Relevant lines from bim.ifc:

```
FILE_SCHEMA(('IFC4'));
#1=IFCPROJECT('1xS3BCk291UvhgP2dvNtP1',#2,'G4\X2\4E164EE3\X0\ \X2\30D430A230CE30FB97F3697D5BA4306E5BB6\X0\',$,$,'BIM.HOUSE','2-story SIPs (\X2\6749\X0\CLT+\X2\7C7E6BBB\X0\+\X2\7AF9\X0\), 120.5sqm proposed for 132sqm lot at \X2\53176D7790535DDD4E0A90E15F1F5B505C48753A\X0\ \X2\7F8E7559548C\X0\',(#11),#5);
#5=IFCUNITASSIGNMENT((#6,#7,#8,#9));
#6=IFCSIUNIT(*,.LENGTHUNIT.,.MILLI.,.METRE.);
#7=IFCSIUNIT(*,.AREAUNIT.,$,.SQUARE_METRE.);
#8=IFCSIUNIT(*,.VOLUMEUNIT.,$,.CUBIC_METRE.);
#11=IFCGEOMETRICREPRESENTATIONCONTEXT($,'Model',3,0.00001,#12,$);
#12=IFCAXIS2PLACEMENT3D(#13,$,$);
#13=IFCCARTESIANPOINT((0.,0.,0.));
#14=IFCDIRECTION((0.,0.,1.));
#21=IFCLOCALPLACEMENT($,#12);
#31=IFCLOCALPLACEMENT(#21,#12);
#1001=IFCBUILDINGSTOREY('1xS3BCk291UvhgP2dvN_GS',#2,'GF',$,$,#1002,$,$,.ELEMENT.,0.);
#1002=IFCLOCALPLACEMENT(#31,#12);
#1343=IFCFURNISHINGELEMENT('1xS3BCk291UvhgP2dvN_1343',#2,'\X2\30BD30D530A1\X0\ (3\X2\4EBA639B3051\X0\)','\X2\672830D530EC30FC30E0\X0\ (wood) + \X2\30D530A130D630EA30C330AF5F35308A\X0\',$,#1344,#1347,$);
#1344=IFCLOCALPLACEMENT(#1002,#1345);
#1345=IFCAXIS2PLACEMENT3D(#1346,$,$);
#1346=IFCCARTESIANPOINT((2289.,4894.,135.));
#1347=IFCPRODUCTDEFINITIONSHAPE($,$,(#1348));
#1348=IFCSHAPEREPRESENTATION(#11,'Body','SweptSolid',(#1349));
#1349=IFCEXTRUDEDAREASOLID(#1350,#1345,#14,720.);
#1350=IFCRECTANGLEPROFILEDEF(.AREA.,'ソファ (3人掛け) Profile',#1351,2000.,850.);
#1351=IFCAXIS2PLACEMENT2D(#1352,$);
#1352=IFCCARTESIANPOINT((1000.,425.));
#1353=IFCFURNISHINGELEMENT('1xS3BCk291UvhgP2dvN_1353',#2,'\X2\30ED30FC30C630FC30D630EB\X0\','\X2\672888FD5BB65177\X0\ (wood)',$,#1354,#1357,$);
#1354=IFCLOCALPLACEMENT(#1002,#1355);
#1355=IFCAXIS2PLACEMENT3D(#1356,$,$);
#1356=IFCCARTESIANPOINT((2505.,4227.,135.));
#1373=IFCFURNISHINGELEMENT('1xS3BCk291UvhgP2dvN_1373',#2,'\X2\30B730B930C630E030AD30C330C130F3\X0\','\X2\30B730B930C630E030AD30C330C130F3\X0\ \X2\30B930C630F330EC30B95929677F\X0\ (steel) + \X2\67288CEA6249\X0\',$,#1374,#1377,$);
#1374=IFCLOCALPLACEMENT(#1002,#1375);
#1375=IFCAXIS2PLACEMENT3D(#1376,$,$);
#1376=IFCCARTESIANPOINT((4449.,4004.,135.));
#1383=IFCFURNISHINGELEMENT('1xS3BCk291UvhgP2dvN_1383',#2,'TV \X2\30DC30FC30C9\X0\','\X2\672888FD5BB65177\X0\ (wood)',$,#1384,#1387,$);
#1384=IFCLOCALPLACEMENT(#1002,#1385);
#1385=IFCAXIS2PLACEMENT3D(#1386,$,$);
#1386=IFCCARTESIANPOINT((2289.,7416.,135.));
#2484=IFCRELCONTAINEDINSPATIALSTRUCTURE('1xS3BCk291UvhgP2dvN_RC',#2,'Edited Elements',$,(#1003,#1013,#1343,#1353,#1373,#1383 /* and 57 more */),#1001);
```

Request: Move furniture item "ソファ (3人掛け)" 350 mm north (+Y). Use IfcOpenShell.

```python
import ifcopenshell
import ifcopenshell.api.geometry
import ifcopenshell.util.placement
import ifcopenshell.util.unit

model = ifcopenshell.open("bim.ifc")
unit_scale = ifcopenshell.util.unit.calculate_unit_scale(model)

item = model.by_guid("1xS3BCk291UvhgP2dvN_1343")
matrix = ifcopenshell.util.placement.get_local_placement(item.ObjectPlacement)
matrix[1, 3] += 0.35 / unit_scale
ifcopenshell.api.geometry.edit_object_placement(model, product=item, matrix=matrix, is_si=False)

print(ifcopenshell.util.placement.get_local_placement(item.ObjectPlacement).round(3) + 0.0)

model.write("bim_rev.ifc")
```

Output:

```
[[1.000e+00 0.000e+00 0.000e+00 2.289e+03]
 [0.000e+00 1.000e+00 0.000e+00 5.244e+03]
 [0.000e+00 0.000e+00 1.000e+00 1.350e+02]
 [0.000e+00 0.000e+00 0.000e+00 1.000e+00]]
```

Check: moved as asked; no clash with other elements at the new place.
